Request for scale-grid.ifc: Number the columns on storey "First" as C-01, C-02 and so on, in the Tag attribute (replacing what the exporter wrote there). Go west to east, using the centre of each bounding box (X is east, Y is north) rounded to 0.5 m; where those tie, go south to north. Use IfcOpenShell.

First a look at what the model holds.

```python
import ifcopenshell
import ifcopenshell.util.element
import ifcopenshell.util.placement

model = ifcopenshell.open("scale-grid.ifc")
print(model.schema)
storey = next(s for s in model.by_type("IfcBuildingStorey") if s.Name == "First")
columns = [e for e in ifcopenshell.util.element.get_decomposition(storey) if e.is_a("IfcColumn")]
for e in sorted(columns, key=lambda e: e.id()):
    origin = ifcopenshell.util.placement.get_local_placement(e.ObjectPlacement)[:3, 3]
    print(e.id(), e.Tag, e.Name, origin.round(2) + 0.0, sep=" | ")
```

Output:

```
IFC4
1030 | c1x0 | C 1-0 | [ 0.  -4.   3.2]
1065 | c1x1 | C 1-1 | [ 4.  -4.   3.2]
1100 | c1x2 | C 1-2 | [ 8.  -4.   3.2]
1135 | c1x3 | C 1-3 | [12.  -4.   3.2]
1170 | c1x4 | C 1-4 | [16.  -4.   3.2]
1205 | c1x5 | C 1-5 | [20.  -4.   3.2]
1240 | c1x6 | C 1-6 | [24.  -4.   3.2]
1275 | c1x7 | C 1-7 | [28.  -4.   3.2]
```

```python
import ifcopenshell
import ifcopenshell.geom
import ifcopenshell.util.element
import ifcopenshell.util.shape

model = ifcopenshell.open("scale-grid.ifc")
settings = ifcopenshell.geom.settings()
settings.set("use-world-coords", True)


def centre(element):
    shape = ifcopenshell.geom.create_shape(settings, element)
    return ifcopenshell.util.shape.get_bbox_centroid(shape.geometry)


storey = next(s for s in model.by_type("IfcBuildingStorey") if s.Name == "First")
columns = [e for e in ifcopenshell.util.element.get_decomposition(storey) if e.is_a("IfcColumn")]

# Insertion points can sit at a corner or the storey origin, so sort by the geometry (in metres).
centres = {e: centre(e) for e in columns}
columns.sort(key=lambda e: (round(centres[e][0] / 0.5), centres[e][1]))

for i, e in enumerate(columns, start=1):
    number = f"C-{i:02d}"
    e.Tag = number
    print(e.id(), number)

model.write("scale-grid_edited.ifc")
```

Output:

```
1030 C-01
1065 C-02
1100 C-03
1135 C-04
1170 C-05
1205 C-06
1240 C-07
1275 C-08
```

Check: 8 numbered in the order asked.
